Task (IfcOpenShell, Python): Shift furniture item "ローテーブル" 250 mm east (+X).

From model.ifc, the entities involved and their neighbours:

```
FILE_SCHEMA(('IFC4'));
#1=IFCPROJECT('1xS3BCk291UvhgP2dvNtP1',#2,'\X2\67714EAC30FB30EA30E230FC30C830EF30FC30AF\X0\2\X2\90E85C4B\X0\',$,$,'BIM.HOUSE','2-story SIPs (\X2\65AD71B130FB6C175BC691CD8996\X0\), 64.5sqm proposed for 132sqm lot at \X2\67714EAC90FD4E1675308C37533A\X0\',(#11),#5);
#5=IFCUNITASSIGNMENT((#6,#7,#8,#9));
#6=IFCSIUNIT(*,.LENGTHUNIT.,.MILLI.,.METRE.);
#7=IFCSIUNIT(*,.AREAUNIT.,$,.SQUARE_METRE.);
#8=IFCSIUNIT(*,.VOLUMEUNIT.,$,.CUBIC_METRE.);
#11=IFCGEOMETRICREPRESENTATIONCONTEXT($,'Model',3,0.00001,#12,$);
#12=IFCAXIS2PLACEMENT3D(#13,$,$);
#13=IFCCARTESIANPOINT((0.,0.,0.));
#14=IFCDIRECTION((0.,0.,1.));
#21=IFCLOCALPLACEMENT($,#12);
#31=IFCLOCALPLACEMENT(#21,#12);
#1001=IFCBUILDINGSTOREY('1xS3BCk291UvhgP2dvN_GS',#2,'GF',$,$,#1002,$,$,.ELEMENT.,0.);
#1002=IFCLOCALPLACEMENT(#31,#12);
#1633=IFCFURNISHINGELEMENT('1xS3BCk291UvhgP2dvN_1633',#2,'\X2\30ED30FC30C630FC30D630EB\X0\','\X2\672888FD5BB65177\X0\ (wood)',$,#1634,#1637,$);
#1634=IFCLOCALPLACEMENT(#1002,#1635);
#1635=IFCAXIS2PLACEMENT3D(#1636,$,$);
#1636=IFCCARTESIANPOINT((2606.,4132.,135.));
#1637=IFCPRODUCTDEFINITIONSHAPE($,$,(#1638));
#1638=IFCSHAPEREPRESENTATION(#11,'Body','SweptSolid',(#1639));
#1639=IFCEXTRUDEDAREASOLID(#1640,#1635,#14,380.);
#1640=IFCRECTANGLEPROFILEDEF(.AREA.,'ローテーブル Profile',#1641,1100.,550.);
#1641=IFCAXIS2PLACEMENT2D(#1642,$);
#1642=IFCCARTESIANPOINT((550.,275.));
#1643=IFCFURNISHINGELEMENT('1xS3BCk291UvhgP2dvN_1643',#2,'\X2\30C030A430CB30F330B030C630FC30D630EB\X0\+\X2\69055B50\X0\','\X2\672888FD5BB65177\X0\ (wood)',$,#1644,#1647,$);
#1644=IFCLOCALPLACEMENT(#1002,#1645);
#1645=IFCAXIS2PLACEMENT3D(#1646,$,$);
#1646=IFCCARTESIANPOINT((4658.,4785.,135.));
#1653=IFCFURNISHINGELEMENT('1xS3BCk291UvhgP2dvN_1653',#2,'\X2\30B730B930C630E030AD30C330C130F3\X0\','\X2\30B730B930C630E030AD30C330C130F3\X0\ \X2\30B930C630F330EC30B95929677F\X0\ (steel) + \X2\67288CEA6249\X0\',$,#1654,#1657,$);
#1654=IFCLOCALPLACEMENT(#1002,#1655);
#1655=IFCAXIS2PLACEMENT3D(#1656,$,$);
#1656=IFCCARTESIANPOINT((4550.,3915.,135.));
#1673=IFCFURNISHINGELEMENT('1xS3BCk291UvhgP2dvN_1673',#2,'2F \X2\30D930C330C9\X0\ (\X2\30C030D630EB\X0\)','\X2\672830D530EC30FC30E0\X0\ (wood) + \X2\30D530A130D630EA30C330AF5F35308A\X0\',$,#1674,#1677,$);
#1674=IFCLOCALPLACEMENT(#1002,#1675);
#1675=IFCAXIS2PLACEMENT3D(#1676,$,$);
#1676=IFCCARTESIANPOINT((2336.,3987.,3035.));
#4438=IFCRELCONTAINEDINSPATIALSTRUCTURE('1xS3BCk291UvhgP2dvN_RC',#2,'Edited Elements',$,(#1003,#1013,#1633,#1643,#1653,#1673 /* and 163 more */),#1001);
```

```python
import ifcopenshell
import ifcopenshell.api.geometry
import ifcopenshell.util.placement
import ifcopenshell.util.unit

model = ifcopenshell.open("model.ifc")
unit_scale = ifcopenshell.util.unit.calculate_unit_scale(model)

item = model.by_guid("1xS3BCk291UvhgP2dvN_1633")
matrix = ifcopenshell.util.placement.get_local_placement(item.ObjectPlacement)
matrix[0, 3] += 0.25 / unit_scale
ifcopenshell.api.geometry.edit_object_placement(model, product=item, matrix=matrix, is_si=False)

print(ifcopenshell.util.placement.get_local_placement(item.ObjectPlacement).round(3) + 0.0)

model.write("model_v2.ifc")
```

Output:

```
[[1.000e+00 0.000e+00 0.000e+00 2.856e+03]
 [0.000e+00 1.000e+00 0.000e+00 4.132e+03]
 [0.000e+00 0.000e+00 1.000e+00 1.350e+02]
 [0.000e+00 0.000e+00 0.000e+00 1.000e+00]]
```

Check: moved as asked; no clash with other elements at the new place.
